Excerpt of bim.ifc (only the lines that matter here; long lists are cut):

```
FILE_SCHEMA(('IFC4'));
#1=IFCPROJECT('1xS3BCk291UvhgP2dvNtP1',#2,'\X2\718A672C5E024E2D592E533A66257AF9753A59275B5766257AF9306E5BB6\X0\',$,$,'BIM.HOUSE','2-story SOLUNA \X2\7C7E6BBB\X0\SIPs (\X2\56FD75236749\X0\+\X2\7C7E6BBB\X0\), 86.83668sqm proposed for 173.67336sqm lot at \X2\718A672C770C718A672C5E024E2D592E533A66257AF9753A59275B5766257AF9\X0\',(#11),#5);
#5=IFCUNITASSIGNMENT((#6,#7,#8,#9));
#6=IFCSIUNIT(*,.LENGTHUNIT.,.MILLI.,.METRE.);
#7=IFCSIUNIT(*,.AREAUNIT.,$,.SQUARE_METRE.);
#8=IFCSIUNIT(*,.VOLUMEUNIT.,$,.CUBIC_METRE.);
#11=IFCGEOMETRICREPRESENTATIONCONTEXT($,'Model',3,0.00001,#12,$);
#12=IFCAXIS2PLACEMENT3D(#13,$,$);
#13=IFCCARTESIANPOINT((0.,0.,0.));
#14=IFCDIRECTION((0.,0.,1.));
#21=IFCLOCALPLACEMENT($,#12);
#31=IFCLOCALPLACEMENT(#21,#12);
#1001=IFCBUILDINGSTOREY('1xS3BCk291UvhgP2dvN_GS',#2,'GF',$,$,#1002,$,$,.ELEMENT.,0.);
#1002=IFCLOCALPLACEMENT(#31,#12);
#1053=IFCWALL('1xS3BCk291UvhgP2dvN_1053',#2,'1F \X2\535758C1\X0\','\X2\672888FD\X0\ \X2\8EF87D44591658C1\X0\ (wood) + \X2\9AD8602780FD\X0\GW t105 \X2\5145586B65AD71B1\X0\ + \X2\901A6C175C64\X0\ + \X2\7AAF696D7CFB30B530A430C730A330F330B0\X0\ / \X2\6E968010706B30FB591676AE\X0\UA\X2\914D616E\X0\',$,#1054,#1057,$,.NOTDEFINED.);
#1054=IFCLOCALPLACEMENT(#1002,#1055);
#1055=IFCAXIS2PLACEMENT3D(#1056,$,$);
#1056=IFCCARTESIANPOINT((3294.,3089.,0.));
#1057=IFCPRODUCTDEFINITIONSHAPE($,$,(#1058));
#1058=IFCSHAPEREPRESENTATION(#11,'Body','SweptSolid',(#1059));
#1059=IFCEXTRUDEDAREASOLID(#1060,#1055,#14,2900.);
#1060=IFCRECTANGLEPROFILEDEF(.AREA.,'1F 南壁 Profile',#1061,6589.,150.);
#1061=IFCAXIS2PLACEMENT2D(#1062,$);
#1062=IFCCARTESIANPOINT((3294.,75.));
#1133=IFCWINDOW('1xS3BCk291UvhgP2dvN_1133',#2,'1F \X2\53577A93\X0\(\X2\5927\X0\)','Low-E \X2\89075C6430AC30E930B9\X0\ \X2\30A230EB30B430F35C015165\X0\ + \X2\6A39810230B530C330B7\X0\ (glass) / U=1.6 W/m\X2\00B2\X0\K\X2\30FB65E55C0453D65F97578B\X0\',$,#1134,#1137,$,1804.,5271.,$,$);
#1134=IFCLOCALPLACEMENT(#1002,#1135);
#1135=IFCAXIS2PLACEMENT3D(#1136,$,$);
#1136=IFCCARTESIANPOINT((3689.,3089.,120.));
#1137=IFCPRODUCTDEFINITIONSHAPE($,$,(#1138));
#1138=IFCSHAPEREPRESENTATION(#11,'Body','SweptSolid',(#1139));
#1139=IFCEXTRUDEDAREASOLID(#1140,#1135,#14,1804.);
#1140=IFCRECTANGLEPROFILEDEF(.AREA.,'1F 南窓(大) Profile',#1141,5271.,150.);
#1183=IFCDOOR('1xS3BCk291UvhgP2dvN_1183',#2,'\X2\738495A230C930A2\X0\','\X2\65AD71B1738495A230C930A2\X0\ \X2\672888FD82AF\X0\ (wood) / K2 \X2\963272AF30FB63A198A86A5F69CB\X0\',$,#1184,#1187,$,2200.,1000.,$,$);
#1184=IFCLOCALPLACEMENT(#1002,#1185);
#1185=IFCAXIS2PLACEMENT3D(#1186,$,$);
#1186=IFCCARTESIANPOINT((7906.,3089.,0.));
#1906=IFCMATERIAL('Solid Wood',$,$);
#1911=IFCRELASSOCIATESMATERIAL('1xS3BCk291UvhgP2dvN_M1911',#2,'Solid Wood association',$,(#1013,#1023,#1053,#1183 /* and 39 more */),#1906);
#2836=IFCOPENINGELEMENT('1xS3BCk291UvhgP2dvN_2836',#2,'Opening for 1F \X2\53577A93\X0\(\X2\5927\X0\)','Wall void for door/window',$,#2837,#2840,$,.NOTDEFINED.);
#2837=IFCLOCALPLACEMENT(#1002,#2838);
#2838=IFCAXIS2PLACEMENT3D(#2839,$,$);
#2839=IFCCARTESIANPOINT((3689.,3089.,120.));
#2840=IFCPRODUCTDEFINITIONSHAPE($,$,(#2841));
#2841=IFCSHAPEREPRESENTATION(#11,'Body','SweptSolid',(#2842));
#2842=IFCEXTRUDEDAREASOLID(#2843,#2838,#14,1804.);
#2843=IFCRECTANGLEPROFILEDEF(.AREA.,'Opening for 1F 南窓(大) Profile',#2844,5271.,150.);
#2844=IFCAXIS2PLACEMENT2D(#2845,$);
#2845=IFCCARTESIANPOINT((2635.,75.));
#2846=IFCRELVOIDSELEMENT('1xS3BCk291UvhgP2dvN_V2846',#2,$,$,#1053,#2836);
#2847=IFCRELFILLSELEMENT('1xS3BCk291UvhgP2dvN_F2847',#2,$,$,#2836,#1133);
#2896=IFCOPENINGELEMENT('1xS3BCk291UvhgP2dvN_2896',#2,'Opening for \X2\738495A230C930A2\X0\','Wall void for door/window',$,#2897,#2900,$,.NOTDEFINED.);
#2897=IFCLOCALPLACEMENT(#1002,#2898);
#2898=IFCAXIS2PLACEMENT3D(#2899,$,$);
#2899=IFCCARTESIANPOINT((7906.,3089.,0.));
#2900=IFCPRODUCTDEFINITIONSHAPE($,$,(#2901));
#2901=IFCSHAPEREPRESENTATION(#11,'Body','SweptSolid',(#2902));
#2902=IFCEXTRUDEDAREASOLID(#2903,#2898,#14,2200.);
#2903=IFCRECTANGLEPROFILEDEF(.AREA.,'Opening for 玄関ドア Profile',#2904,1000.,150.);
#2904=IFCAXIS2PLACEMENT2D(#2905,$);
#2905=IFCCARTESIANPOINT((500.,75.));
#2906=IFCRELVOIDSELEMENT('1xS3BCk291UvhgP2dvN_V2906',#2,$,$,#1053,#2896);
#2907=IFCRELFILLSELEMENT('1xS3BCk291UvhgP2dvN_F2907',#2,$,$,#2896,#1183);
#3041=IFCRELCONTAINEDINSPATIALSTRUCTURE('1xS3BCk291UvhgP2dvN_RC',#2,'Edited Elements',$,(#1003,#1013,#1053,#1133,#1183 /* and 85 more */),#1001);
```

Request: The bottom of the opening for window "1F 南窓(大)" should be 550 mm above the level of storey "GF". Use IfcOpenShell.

```python
import numpy as np
import ifcopenshell
import ifcopenshell.api.geometry
import ifcopenshell.geom
import ifcopenshell.util.element
import ifcopenshell.util.placement
import ifcopenshell.util.shape
import ifcopenshell.util.unit

model = ifcopenshell.open("bim.ifc")
unit_scale = ifcopenshell.util.unit.calculate_unit_scale(model)

window = model.by_id(1133)
opening = window.FillsVoids[0].RelatingOpeningElement
storey = ifcopenshell.util.element.get_container(window, ifc_class="IfcBuildingStorey")
level = ifcopenshell.util.placement.get_local_placement(storey.ObjectPlacement)[2, 3]

# The opening's origin need not be at the sill, so measure its lowest point.
shape = ifcopenshell.geom.create_shape(ifcopenshell.geom.settings(), opening)
bottom = ifcopenshell.util.shape.get_shape_bottom_elevation(shape, shape.geometry) / unit_scale
dz = level + 0.55 / unit_scale - bottom

shift = np.array([0.0, 0.0, dz])
# The window is not placed relative to its opening, so move both.
for product in (opening, window):
    matrix = ifcopenshell.util.placement.get_local_placement(product.ObjectPlacement)
    matrix[:3, 3] += shift
    ifcopenshell.api.geometry.edit_object_placement(model, product=product, matrix=matrix, is_si=False)

print(f"moved by {dz * unit_scale:+.3f} m")

model.write("bim-out.ifc")
```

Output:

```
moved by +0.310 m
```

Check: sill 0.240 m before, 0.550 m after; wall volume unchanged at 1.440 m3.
